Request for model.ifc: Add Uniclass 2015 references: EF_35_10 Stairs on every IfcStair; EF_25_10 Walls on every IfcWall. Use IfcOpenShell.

First a look at what the model holds.

```python
import ifcopenshell

model = ifcopenshell.open("model.ifc")
print(model.schema)
print("classifications:", [c.Name for c in model.by_type("IfcClassification")])
for ifc_class in ("IfcDoor", "IfcRoof", "IfcStair", "IfcWall", "IfcWindow"):
    print(ifc_class, len(model.by_type(ifc_class)))
```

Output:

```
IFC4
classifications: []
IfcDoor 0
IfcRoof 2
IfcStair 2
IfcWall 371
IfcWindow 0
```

```python
import ifcopenshell
import ifcopenshell.api.classification

model = ifcopenshell.open("model.ifc")

system = ifcopenshell.api.classification.add_classification(model, classification="Uniclass 2015")

codes = {
    "IfcStair": ("EF_35_10", "Stairs"),
    "IfcWall": ("EF_25_10", "Walls"),
}
for ifc_class, (code, name) in codes.items():
    products = model.by_type(ifc_class)
    ifcopenshell.api.classification.add_reference(
        model, products=products, classification=system, identification=code, name=name
    )
    print(code, len(products))

model.write("model_rev.ifc")
```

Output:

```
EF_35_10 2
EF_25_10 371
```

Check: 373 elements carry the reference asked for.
